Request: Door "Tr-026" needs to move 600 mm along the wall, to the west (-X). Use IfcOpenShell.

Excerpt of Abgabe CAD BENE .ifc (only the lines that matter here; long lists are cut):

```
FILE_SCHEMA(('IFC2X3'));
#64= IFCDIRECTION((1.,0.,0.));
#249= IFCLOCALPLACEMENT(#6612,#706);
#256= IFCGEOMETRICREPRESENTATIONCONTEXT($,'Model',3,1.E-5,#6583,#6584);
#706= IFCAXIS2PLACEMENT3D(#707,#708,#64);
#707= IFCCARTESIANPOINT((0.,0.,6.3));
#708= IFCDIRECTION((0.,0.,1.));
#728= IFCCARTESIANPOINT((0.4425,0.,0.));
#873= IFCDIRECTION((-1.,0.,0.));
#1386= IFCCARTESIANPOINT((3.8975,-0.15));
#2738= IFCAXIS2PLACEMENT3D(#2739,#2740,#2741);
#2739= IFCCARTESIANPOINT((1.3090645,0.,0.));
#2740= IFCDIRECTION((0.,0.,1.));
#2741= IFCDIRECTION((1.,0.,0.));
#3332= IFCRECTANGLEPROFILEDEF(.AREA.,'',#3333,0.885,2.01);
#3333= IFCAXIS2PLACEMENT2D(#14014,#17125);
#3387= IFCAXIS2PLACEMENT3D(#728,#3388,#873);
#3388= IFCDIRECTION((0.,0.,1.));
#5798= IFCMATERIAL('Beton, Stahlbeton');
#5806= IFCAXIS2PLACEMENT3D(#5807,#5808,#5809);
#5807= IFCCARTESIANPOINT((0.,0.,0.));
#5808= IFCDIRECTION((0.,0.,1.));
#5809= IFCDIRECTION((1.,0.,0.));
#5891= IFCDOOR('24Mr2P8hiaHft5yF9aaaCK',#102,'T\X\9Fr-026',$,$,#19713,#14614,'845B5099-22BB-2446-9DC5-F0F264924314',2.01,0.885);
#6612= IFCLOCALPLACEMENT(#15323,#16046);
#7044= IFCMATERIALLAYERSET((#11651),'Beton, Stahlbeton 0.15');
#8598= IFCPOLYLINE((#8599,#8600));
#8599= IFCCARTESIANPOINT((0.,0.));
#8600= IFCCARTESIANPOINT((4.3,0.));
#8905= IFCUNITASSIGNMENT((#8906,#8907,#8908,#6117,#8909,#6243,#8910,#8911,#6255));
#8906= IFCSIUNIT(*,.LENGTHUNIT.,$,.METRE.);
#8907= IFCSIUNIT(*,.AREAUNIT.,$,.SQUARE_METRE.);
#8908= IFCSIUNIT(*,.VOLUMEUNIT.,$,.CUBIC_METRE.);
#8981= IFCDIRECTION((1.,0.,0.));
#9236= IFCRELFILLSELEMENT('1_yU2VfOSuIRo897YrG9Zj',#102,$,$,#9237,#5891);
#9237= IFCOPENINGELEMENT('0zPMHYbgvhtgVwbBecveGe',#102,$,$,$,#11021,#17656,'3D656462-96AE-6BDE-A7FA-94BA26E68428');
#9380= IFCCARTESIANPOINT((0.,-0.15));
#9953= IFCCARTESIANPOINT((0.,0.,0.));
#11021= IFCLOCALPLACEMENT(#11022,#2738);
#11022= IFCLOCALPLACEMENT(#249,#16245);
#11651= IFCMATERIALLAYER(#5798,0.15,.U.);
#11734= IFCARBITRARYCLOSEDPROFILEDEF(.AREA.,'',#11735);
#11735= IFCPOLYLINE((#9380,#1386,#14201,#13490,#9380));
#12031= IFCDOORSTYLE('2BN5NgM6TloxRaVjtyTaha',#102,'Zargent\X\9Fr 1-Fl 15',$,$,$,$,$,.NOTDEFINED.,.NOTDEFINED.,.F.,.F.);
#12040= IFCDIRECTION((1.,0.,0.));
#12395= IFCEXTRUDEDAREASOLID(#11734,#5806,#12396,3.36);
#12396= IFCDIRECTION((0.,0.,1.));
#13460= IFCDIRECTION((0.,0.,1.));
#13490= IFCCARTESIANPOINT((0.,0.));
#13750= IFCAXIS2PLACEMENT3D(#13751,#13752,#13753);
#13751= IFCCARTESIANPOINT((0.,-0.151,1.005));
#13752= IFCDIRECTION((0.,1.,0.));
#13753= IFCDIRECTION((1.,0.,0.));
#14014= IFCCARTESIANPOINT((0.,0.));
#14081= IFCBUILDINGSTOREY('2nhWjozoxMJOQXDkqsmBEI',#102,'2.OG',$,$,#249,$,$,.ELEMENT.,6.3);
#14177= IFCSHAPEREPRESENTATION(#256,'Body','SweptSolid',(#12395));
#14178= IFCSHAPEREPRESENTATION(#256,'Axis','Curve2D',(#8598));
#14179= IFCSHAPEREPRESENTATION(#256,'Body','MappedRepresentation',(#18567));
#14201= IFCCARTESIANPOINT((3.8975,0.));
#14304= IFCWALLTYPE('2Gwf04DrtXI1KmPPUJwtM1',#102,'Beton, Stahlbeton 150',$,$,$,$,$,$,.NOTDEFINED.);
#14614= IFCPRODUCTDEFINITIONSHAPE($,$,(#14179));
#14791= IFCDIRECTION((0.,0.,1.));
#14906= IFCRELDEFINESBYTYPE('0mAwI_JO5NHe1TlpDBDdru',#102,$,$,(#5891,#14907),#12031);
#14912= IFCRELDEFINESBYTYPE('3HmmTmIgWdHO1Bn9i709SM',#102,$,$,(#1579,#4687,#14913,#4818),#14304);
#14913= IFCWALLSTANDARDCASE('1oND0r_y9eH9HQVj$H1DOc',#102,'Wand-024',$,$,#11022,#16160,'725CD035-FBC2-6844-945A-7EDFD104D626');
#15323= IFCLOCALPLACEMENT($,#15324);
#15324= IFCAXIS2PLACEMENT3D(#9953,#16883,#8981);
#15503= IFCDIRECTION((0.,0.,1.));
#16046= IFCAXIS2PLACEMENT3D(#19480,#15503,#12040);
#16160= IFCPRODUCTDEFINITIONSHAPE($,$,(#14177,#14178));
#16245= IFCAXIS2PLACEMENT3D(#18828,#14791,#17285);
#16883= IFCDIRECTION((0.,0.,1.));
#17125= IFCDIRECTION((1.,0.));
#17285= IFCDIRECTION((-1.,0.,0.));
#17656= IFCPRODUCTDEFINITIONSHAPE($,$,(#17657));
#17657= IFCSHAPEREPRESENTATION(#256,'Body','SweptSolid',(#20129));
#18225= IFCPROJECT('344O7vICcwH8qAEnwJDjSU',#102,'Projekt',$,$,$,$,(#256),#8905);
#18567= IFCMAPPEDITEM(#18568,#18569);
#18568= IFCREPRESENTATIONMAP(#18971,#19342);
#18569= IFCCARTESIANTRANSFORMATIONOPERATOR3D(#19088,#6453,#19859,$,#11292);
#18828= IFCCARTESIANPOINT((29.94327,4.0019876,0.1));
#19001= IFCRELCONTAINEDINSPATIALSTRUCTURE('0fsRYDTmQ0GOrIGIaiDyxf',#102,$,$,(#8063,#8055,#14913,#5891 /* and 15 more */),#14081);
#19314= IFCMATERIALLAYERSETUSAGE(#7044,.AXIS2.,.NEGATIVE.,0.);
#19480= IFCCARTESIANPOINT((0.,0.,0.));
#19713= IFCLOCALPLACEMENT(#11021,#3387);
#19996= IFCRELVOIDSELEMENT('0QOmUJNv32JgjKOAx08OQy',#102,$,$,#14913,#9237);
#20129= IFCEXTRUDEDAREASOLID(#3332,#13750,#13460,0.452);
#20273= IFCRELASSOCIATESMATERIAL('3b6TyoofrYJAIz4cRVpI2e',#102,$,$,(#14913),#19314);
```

```python
import ifcopenshell
import ifcopenshell.api.geometry
import ifcopenshell.util.placement

model = ifcopenshell.open("Abgabe CAD BENE .ifc")

door = model.by_id(5891)
opening = door.FillsVoids[0].RelatingOpeningElement
wall = opening.VoidsElements[0].RelatingBuildingElement

wall_matrix = ifcopenshell.util.placement.get_local_placement(wall.ObjectPlacement)
shift = wall_matrix[:3, 0] * 0.6
before = ifcopenshell.util.placement.get_local_placement(door.ObjectPlacement)[:3, 3].copy()

# The door is placed relative to its opening, so it follows when the opening moves.
matrix = ifcopenshell.util.placement.get_local_placement(opening.ObjectPlacement)
matrix[:3, 3] += shift
ifcopenshell.api.geometry.edit_object_placement(
    model, product=opening, matrix=matrix, is_si=False, should_transform_children=True
)

after = ifcopenshell.util.placement.get_local_placement(door.ObjectPlacement)[:3, 3]
print("door moved by", (after - before).round(3) + 0.0)

model.write("Abgabe CAD BENE _edited.ifc")
```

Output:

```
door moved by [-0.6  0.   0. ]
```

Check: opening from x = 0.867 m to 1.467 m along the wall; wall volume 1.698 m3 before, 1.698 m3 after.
